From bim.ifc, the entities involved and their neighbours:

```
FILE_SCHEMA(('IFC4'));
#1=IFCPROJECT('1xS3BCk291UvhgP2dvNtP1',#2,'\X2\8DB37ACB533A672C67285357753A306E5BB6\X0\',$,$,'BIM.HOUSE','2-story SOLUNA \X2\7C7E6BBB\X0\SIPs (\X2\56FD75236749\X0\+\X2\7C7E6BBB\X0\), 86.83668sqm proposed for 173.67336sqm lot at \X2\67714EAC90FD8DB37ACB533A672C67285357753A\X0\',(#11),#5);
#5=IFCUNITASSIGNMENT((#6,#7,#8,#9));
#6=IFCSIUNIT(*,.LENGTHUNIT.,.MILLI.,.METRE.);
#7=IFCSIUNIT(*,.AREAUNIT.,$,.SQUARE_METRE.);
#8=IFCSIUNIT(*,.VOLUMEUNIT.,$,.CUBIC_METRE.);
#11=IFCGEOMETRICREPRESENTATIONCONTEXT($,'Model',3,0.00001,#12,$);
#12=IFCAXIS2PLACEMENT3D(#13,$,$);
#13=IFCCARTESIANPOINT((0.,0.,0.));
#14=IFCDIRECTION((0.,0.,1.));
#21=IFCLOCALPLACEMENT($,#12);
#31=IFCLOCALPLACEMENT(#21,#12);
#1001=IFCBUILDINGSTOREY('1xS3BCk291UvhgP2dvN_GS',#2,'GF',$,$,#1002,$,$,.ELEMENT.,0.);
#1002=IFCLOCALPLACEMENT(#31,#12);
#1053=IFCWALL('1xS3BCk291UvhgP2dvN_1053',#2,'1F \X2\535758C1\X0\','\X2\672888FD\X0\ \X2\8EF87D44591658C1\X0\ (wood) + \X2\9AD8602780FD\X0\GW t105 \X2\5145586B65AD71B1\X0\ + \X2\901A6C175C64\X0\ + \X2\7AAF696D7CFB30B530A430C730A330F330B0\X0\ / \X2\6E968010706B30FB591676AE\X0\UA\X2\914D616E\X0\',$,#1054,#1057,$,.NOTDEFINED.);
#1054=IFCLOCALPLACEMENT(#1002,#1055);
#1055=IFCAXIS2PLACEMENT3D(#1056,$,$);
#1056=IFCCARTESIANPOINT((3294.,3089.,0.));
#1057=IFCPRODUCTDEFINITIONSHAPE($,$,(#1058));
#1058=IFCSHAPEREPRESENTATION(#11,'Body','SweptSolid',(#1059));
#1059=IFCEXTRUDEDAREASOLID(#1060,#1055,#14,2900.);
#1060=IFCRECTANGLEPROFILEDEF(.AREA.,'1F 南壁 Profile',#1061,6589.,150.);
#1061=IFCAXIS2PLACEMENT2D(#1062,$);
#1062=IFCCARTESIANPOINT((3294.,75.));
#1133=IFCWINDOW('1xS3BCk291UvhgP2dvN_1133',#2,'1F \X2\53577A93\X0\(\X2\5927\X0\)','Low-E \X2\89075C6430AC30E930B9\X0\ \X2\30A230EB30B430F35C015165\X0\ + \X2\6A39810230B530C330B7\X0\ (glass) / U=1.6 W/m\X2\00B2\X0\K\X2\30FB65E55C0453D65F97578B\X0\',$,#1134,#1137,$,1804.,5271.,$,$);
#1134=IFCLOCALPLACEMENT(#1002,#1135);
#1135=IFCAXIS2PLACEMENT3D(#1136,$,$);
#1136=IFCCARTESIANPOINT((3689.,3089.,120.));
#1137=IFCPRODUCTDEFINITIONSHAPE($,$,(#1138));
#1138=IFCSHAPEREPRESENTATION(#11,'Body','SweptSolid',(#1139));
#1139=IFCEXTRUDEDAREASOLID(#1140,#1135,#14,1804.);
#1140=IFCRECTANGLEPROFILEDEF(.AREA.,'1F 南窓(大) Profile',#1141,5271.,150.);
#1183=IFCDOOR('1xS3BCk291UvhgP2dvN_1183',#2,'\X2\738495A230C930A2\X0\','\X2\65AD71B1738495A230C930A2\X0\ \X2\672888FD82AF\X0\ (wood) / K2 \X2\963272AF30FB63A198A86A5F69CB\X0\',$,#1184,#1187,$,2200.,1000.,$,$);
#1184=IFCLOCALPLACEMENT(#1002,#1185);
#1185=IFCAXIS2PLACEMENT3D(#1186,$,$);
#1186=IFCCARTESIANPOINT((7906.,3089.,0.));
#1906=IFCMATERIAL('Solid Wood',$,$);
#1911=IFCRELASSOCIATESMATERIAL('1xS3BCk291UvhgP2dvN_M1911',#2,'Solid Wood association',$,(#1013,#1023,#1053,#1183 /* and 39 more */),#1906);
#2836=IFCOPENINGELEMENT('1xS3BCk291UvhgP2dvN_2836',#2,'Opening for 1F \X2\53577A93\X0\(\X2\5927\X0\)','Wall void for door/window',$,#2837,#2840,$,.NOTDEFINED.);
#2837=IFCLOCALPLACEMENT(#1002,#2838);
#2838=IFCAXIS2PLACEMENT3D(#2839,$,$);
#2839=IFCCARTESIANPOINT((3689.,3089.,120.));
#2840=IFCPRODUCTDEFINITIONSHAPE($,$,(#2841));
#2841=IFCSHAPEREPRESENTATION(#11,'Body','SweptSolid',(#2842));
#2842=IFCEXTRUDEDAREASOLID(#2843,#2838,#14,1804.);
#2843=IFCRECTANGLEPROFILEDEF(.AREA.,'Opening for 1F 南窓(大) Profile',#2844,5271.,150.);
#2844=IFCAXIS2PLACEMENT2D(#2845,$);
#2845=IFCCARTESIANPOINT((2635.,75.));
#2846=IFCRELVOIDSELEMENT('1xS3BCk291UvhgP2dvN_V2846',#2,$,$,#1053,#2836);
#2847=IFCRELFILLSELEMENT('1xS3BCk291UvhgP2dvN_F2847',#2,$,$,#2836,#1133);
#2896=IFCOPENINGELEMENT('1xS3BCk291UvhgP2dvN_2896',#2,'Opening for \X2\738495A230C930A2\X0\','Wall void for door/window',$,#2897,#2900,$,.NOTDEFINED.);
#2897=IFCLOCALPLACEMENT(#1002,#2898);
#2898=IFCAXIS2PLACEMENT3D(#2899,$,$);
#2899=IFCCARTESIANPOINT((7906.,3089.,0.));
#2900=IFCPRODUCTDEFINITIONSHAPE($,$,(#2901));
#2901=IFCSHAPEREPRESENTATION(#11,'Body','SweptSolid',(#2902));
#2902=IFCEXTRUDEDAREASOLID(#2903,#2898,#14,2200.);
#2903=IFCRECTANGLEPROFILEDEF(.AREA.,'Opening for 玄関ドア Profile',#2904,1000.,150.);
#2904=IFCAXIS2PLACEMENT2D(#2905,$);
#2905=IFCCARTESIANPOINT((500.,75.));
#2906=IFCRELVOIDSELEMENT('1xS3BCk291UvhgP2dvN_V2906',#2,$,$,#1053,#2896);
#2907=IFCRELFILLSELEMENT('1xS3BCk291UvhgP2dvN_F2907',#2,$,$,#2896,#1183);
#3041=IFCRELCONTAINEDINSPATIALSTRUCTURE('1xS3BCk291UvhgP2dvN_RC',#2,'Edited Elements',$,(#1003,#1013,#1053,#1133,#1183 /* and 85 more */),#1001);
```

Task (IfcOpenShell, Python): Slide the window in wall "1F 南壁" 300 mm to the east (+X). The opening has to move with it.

```python
import ifcopenshell
import ifcopenshell.api.geometry
import ifcopenshell.util.placement

model = ifcopenshell.open("bim.ifc")

window = model.by_guid("1xS3BCk291UvhgP2dvN_1133")
opening = window.FillsVoids[0].RelatingOpeningElement
wall = opening.VoidsElements[0].RelatingBuildingElement

wall_matrix = ifcopenshell.util.placement.get_local_placement(wall.ObjectPlacement)
shift = wall_matrix[:3, 0] * 300.0
before = ifcopenshell.util.placement.get_local_placement(window.ObjectPlacement)[:3, 3].copy()

# The window is not placed relative to its opening, so move both.
for product in (opening, window):
    matrix = ifcopenshell.util.placement.get_local_placement(product.ObjectPlacement)
    matrix[:3, 3] += shift
    ifcopenshell.api.geometry.edit_object_placement(model, product=product, matrix=matrix, is_si=False)

after = ifcopenshell.util.placement.get_local_placement(window.ObjectPlacement)[:3, 3]
print("window moved by", (after - before).round(3) + 0.0)

model.write("bim_v2.ifc")
```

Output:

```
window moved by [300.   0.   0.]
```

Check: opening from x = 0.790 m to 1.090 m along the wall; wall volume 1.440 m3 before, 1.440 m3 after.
